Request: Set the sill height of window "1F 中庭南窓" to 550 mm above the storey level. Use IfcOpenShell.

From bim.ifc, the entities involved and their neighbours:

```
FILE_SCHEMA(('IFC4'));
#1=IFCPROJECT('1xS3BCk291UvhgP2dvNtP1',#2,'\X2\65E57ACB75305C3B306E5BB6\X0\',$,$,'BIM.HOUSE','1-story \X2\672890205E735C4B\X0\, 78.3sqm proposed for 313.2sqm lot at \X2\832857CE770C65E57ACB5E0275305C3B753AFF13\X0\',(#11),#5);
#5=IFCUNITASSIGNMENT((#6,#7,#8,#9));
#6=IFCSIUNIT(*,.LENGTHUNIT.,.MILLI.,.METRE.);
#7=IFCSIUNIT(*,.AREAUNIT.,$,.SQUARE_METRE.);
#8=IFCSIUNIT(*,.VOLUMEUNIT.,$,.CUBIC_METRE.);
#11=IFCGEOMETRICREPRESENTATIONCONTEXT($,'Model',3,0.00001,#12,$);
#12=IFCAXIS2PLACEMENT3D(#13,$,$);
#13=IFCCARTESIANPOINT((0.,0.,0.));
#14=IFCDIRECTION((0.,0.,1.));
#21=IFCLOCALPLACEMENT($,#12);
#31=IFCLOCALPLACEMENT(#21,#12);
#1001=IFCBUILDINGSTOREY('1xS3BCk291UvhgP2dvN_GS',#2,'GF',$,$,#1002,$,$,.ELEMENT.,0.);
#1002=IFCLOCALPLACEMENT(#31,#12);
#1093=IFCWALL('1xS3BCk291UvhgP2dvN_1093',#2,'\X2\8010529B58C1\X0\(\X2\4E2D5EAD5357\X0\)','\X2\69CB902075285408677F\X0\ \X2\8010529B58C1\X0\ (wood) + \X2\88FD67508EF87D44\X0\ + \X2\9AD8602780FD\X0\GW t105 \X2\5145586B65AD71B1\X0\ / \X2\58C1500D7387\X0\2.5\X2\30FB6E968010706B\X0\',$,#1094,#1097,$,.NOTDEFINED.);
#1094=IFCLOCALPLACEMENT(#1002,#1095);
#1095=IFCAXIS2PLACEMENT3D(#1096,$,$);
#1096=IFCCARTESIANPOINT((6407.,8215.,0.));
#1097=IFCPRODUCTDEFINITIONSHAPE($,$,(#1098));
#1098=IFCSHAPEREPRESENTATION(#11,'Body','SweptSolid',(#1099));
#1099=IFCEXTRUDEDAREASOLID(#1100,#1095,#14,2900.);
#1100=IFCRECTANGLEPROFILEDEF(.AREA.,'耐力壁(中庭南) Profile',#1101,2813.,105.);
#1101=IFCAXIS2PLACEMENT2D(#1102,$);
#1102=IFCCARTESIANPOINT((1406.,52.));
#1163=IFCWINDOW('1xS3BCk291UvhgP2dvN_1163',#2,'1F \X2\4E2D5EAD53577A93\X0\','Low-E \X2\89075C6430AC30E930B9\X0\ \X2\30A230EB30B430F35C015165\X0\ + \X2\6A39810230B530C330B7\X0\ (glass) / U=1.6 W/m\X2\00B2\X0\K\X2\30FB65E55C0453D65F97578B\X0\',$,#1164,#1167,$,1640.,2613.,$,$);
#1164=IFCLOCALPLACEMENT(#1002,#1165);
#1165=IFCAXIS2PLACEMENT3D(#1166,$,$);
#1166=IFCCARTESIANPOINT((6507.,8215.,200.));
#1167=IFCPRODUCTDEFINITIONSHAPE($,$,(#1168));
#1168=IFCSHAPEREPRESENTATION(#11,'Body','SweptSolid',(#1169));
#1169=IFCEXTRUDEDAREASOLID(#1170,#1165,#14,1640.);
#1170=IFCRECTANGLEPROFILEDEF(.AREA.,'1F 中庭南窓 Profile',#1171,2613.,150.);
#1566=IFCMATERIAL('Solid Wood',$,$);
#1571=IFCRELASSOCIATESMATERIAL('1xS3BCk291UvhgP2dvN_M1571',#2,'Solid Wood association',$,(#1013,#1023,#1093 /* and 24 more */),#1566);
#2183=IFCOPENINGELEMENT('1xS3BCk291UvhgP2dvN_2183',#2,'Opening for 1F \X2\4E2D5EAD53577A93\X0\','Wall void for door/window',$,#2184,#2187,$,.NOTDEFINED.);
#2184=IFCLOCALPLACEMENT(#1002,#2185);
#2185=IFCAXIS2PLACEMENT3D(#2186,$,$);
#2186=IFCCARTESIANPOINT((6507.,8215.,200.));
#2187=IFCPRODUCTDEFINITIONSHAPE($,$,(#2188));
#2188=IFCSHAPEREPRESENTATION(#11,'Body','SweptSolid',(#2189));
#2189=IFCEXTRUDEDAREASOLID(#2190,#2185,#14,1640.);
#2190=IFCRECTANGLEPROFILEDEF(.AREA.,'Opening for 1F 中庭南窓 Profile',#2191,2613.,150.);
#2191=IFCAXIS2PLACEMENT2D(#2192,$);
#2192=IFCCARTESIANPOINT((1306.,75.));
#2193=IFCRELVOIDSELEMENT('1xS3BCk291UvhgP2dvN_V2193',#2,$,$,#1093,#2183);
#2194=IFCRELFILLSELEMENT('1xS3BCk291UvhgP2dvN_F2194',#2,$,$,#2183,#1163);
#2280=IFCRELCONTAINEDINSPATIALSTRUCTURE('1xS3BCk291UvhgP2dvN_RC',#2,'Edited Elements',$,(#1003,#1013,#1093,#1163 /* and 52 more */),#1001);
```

```python
import numpy as np
import ifcopenshell
import ifcopenshell.api.geometry
import ifcopenshell.geom
import ifcopenshell.util.element
import ifcopenshell.util.placement
import ifcopenshell.util.shape
import ifcopenshell.util.unit

model = ifcopenshell.open("bim.ifc")
unit_scale = ifcopenshell.util.unit.calculate_unit_scale(model)

window = model.by_id(1163)
opening = window.FillsVoids[0].RelatingOpeningElement
storey = ifcopenshell.util.element.get_container(window, ifc_class="IfcBuildingStorey")
level = ifcopenshell.util.placement.get_local_placement(storey.ObjectPlacement)[2, 3]

# The opening's origin need not be at the sill, so measure its lowest point.
shape = ifcopenshell.geom.create_shape(ifcopenshell.geom.settings(), opening)
bottom = ifcopenshell.util.shape.get_shape_bottom_elevation(shape, shape.geometry) / unit_scale
dz = level + 550.0 - bottom

shift = np.array([0.0, 0.0, dz])
# The window is not placed relative to its opening, so move both.
for product in (opening, window):
    matrix = ifcopenshell.util.placement.get_local_placement(product.ObjectPlacement)
    matrix[:3, 3] += shift
    ifcopenshell.api.geometry.edit_object_placement(model, product=product, matrix=matrix, is_si=False)

print(f"moved by {dz * unit_scale:+.3f} m")

model.write("bim_updated.ifc")
```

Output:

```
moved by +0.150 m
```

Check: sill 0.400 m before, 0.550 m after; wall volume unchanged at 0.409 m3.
